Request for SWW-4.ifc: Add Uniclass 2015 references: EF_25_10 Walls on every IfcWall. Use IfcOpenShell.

First a look at what the model holds.

```python
import ifcopenshell

model = ifcopenshell.open("SWW-4.ifc")
print(model.schema)
print("classifications:", [c.Name for c in model.by_type("IfcClassification")])
for ifc_class in ("IfcDoor", "IfcRoof", "IfcStair", "IfcWall", "IfcWindow"):
    print(ifc_class, len(model.by_type(ifc_class)))
```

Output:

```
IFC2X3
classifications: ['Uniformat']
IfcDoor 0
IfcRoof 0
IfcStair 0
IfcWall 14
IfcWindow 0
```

```python
import ifcopenshell
import ifcopenshell.api.classification

model = ifcopenshell.open("SWW-4.ifc")

# IFC2X3 requires Source and Edition and has no link from the project to the system.
system = model.create_entity("IfcClassification", Source="NBS", Edition="2015", Name="Uniclass 2015")

codes = {
    "IfcWall": ("EF_25_10", "Walls"),
}
for ifc_class, (code, name) in codes.items():
    products = model.by_type(ifc_class)
    ifcopenshell.api.classification.add_reference(
        model, products=products, classification=system, identification=code, name=name
    )
    print(code, len(products))

model.write("SWW-4-out.ifc")
```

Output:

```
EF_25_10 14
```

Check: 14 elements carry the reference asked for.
